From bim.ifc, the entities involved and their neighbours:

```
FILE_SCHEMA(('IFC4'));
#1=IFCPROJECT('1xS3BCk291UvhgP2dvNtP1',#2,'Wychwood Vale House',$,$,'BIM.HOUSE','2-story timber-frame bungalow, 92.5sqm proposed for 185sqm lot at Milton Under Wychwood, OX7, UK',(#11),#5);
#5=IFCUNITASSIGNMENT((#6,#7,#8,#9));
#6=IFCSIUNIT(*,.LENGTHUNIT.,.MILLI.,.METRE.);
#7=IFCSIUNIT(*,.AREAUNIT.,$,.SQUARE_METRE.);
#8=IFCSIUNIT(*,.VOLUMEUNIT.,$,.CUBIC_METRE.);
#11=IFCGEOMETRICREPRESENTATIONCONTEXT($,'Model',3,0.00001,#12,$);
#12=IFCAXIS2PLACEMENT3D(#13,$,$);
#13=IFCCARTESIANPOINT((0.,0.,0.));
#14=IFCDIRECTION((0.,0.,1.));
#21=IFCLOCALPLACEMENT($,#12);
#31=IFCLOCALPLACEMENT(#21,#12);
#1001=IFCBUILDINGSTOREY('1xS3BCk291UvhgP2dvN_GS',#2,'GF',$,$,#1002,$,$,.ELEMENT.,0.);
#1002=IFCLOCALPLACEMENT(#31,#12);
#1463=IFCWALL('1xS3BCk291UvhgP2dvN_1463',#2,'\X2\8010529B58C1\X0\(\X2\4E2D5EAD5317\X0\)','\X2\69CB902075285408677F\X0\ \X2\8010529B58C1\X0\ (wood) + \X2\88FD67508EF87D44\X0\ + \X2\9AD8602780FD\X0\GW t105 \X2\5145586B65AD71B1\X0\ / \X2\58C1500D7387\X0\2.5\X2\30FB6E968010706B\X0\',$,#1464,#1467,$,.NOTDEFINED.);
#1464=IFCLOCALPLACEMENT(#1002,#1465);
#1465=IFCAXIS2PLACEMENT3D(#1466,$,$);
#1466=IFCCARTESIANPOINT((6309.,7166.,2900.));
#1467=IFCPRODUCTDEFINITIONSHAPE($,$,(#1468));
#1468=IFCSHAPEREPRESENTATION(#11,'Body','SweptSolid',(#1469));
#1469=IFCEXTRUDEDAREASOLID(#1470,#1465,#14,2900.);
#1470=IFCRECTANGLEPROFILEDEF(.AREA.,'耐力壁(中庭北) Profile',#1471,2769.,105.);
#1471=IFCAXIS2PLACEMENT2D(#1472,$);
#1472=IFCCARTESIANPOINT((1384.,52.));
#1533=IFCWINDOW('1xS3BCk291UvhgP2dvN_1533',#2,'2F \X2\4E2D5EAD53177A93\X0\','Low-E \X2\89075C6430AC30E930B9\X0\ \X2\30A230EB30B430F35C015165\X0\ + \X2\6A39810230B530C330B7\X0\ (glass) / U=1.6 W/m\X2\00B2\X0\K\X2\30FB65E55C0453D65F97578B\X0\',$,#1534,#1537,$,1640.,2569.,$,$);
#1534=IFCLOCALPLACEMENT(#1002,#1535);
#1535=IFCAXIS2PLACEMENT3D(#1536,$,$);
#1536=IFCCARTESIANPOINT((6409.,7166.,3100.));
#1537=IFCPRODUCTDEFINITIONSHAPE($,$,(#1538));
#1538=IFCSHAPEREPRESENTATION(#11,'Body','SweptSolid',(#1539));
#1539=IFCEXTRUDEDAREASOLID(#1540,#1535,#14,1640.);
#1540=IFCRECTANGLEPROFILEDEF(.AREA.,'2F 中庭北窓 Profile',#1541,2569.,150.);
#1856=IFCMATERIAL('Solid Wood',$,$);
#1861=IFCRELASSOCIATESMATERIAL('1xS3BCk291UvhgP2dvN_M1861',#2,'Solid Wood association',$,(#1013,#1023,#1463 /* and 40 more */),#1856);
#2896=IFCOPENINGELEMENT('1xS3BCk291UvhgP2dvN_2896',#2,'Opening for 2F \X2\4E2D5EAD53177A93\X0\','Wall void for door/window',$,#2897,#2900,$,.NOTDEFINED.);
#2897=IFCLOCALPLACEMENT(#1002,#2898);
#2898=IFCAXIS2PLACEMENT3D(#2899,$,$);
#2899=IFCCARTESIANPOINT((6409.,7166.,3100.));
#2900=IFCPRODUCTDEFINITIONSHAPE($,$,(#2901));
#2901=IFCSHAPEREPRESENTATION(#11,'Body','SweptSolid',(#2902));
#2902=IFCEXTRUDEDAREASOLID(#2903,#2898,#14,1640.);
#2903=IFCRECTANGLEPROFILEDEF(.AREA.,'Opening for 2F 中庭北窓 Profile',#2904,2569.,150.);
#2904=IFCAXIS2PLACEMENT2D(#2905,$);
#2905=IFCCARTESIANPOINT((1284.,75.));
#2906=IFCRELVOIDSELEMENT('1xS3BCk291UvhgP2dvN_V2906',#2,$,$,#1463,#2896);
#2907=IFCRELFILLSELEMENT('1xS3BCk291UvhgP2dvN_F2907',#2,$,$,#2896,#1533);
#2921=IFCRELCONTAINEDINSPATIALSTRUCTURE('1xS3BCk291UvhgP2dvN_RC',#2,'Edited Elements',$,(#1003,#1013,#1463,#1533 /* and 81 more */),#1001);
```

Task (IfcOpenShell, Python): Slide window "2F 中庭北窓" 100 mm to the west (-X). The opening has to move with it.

```python
import ifcopenshell
import ifcopenshell.api.geometry
import ifcopenshell.util.placement
import ifcopenshell.util.unit

model = ifcopenshell.open("bim.ifc")
unit_scale = ifcopenshell.util.unit.calculate_unit_scale(model)

window = model.by_guid("1xS3BCk291UvhgP2dvN_1533")
opening = window.FillsVoids[0].RelatingOpeningElement
wall = opening.VoidsElements[0].RelatingBuildingElement

wall_matrix = ifcopenshell.util.placement.get_local_placement(wall.ObjectPlacement)
shift = wall_matrix[:3, 0] * -0.1 / unit_scale
before = ifcopenshell.util.placement.get_local_placement(window.ObjectPlacement)[:3, 3].copy()

# The window is not placed relative to its opening, so move both.
for product in (opening, window):
    matrix = ifcopenshell.util.placement.get_local_placement(product.ObjectPlacement)
    matrix[:3, 3] += shift
    ifcopenshell.api.geometry.edit_object_placement(model, product=product, matrix=matrix, is_si=False)

after = ifcopenshell.util.placement.get_local_placement(window.ObjectPlacement)[:3, 3]
print("window moved by", (after - before).round(3) + 0.0)

model.write("bim_updated.ifc")
```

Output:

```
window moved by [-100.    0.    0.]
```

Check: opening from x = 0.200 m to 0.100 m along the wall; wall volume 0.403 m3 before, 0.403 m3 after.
